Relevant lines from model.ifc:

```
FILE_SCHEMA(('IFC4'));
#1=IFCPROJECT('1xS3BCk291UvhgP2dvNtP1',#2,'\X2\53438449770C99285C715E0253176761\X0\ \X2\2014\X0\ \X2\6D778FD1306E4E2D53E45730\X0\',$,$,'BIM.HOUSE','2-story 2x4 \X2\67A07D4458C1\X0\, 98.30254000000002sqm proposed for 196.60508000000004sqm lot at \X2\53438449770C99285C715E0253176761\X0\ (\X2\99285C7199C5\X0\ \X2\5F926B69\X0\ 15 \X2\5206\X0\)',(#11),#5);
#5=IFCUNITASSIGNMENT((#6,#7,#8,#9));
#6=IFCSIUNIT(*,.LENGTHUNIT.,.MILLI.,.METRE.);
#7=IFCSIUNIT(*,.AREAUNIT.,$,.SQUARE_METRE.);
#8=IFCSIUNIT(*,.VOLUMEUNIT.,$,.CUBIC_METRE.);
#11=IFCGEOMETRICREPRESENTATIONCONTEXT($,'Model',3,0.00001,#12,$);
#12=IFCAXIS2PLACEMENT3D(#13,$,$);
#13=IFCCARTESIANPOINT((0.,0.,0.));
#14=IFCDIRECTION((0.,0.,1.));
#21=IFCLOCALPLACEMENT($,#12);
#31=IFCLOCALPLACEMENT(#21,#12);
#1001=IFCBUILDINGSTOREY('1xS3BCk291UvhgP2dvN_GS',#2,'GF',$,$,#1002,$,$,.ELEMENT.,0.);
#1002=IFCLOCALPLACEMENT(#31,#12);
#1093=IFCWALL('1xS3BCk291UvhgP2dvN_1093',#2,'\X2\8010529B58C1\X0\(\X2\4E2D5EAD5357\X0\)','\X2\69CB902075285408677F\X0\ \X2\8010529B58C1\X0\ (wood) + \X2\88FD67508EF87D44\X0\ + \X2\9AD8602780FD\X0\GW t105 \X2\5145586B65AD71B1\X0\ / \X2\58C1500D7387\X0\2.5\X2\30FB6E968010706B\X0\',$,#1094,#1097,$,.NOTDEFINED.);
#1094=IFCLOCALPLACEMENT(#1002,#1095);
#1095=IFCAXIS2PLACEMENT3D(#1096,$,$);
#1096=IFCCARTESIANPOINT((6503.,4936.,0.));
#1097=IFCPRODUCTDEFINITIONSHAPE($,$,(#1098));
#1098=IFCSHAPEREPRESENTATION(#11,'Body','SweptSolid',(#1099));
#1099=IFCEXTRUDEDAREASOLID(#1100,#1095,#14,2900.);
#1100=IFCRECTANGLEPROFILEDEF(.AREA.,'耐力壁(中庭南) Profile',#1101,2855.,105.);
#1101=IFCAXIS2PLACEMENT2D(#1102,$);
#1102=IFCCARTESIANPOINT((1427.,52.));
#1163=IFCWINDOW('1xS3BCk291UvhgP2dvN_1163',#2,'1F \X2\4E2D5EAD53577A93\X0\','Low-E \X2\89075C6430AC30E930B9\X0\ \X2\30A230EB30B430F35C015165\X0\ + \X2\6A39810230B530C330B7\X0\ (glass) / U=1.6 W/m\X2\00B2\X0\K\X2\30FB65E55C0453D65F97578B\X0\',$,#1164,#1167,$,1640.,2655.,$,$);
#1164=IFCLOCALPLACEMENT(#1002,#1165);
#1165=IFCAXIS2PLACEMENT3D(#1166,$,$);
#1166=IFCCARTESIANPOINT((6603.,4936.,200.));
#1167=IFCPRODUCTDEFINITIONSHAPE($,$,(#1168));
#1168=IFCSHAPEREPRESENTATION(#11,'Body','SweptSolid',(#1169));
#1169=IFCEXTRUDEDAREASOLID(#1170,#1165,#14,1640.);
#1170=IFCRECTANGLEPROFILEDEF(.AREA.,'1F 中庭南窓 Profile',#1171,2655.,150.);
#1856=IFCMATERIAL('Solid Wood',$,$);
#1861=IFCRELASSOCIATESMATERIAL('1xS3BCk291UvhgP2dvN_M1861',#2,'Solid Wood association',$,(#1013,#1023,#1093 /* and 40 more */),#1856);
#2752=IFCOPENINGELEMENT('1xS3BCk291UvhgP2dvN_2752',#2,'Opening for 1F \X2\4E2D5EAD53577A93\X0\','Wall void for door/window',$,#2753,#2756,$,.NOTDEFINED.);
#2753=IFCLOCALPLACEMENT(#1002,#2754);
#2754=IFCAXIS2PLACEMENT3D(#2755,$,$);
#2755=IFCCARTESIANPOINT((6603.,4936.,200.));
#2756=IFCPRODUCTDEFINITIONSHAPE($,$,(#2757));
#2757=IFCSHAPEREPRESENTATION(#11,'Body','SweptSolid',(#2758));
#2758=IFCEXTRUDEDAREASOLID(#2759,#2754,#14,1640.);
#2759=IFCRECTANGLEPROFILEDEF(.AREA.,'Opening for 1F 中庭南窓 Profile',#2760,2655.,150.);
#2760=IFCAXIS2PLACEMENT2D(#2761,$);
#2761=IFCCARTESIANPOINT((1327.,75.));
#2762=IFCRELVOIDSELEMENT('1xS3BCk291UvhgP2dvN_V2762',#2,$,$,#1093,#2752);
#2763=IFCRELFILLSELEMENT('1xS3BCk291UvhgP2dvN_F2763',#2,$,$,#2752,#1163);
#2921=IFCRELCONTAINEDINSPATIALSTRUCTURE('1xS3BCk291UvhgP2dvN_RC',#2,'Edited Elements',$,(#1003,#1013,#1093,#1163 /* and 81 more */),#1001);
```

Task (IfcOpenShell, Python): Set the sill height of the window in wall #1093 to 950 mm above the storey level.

```python
import numpy as np
import ifcopenshell
import ifcopenshell.api.geometry
import ifcopenshell.geom
import ifcopenshell.util.element
import ifcopenshell.util.placement
import ifcopenshell.util.shape
import ifcopenshell.util.unit

model = ifcopenshell.open("model.ifc")
unit_scale = ifcopenshell.util.unit.calculate_unit_scale(model)

window = model.by_guid("1xS3BCk291UvhgP2dvN_1163")
opening = window.FillsVoids[0].RelatingOpeningElement
storey = ifcopenshell.util.element.get_container(window, ifc_class="IfcBuildingStorey")
level = ifcopenshell.util.placement.get_local_placement(storey.ObjectPlacement)[2, 3]

# The opening's origin need not be at the sill, so measure its lowest point.
shape = ifcopenshell.geom.create_shape(ifcopenshell.geom.settings(), opening)
bottom = ifcopenshell.util.shape.get_shape_bottom_elevation(shape, shape.geometry) / unit_scale
dz = level + 0.95 / unit_scale - bottom

shift = np.array([0.0, 0.0, dz])
# The window is not placed relative to its opening, so move both.
for product in (opening, window):
    matrix = ifcopenshell.util.placement.get_local_placement(product.ObjectPlacement)
    matrix[:3, 3] += shift
    ifcopenshell.api.geometry.edit_object_placement(model, product=product, matrix=matrix, is_si=False)

print(f"moved by {dz * unit_scale:+.3f} m")

model.write("model_updated.ifc")
```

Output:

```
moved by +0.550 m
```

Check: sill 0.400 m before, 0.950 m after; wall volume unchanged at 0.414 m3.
